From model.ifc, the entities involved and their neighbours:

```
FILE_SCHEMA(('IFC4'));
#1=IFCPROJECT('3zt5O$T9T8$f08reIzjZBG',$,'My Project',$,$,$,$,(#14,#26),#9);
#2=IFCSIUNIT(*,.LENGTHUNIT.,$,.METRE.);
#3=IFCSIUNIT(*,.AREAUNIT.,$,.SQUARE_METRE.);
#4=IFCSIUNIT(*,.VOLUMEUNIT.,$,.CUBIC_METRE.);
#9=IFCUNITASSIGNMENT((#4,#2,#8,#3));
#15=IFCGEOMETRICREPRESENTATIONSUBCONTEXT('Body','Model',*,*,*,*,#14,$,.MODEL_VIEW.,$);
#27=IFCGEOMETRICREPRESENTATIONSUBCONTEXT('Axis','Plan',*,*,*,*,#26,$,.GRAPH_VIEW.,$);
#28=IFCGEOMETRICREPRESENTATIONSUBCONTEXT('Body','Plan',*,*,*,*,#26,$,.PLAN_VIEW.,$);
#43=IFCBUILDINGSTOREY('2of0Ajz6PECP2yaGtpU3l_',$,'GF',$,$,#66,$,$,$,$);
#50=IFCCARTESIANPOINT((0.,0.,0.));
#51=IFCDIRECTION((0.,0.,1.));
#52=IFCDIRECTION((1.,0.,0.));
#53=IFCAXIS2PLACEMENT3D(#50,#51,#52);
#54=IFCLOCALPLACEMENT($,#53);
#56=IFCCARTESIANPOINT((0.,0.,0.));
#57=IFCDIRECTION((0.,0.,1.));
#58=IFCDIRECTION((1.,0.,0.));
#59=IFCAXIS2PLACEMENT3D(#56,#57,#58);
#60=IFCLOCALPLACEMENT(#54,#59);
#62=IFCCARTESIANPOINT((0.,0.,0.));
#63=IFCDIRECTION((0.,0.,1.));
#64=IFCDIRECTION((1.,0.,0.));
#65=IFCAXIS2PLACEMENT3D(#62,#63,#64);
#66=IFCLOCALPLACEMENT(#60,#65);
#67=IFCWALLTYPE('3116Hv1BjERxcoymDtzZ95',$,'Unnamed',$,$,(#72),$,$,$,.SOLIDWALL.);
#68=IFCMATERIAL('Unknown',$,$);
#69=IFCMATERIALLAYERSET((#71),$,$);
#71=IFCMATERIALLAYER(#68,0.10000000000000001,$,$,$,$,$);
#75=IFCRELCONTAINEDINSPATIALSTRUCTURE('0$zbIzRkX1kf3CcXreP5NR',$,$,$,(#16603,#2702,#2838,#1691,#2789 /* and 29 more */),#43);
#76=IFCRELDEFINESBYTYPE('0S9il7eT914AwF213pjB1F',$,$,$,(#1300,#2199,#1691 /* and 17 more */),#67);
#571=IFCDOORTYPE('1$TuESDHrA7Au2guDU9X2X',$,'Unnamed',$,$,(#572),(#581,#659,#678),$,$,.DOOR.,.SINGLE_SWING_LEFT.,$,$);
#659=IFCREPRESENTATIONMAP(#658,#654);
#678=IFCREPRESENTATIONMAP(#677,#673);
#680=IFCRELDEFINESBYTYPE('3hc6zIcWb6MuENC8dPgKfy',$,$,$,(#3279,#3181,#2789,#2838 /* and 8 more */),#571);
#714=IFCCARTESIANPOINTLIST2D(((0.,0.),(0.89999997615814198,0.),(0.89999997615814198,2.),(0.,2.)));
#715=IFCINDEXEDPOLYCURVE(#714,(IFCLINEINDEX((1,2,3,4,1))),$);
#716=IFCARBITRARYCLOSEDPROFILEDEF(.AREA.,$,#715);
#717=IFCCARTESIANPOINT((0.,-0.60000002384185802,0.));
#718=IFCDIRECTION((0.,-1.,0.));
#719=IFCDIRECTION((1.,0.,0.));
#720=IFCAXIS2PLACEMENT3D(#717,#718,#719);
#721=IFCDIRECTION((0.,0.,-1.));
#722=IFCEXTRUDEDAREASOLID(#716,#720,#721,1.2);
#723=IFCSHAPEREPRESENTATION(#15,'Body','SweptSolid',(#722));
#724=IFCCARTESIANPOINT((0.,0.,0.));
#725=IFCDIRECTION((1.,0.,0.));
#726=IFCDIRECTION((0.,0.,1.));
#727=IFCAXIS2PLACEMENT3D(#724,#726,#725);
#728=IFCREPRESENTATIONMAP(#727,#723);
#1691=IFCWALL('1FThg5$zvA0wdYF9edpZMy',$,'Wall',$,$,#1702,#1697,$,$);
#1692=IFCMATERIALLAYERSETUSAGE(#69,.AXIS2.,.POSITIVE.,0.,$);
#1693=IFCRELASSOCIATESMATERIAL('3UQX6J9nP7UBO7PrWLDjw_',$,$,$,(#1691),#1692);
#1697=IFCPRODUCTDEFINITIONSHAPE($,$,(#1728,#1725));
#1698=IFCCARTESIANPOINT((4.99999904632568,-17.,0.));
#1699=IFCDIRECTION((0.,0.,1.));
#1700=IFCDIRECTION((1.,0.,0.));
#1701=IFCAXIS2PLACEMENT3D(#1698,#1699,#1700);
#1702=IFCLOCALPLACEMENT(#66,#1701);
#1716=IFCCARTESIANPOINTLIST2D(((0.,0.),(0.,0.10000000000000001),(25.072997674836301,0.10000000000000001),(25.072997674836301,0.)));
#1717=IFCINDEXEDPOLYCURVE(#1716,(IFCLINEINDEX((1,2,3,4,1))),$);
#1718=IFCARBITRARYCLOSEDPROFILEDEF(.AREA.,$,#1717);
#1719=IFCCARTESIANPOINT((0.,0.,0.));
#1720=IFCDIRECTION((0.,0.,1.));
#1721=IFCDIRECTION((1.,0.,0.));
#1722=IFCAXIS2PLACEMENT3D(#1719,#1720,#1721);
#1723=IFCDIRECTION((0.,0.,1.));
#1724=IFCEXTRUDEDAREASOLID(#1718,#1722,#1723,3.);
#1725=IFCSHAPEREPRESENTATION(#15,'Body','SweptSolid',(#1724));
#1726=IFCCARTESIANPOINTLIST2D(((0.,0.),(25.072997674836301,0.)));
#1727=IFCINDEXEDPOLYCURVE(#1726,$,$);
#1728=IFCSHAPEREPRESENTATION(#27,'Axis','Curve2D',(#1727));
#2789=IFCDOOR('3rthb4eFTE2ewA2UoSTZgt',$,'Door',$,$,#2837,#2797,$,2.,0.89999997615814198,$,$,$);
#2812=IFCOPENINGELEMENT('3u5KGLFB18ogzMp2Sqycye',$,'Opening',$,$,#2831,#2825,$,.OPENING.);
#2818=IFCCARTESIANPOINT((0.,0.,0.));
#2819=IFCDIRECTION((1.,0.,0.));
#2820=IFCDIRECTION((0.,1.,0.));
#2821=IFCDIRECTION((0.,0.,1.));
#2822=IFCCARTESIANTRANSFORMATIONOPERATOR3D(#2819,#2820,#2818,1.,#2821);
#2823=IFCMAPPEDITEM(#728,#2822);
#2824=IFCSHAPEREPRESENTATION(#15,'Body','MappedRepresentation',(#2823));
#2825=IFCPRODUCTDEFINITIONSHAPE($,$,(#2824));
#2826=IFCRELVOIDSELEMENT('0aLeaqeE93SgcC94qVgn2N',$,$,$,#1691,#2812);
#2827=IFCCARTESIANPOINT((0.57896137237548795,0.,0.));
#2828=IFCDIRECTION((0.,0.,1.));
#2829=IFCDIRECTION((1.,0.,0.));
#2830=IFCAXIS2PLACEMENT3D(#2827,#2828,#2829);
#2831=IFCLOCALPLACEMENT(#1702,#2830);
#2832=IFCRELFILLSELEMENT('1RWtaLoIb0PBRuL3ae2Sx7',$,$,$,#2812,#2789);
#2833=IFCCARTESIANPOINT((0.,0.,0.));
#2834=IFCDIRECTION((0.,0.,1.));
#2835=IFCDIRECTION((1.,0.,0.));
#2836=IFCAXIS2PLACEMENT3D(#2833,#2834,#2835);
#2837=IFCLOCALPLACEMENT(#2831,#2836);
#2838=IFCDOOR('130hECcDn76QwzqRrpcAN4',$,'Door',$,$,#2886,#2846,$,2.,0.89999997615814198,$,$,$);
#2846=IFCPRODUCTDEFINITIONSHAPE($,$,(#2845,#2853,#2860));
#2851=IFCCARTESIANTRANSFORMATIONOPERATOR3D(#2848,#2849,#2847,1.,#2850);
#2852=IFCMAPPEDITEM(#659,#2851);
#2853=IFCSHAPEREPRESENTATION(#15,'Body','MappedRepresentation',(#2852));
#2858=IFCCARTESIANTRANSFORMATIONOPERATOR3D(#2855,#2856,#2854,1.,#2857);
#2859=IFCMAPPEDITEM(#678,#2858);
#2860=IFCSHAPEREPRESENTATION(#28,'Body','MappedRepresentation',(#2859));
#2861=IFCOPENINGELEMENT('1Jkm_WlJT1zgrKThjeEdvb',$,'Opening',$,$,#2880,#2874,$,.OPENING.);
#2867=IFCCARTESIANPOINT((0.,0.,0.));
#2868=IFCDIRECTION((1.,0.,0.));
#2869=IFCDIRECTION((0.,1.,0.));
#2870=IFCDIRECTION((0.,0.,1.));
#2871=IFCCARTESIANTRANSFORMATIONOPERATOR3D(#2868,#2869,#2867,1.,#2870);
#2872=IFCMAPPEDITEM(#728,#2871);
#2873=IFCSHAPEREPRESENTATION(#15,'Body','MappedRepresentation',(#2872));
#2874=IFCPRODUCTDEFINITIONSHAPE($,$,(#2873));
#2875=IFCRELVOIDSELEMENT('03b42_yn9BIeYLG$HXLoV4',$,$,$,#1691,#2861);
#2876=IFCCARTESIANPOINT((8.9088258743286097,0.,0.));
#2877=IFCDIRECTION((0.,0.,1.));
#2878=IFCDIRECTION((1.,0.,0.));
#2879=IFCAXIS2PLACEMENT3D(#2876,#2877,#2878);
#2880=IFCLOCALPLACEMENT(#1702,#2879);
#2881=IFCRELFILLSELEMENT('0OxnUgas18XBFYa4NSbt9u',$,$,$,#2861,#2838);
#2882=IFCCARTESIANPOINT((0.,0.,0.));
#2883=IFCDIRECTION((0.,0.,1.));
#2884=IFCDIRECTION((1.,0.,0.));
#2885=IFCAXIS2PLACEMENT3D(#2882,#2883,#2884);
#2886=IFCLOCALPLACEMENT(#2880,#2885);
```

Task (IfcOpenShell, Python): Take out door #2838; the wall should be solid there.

```python
import ifcopenshell
import ifcopenshell.api.feature
import ifcopenshell.api.root
import ifcopenshell.geom
import ifcopenshell.util.shape

model = ifcopenshell.open("model.ifc")
settings = ifcopenshell.geom.settings()


def volume(element):
    """Net volume in cubic metres, openings subtracted."""
    shape = ifcopenshell.geom.create_shape(settings, element)
    return ifcopenshell.util.shape.get_volume(shape.geometry)


door = model.by_guid("130hECcDn76QwzqRrpcAN4")
opening = door.FillsVoids[0].RelatingOpeningElement
wall = opening.VoidsElements[0].RelatingBuildingElement
before = volume(wall)

ifcopenshell.api.root.remove_product(model, product=door)
ifcopenshell.api.feature.remove_feature(model, feature=opening)

after = volume(wall)

print(f"wall volume {before:.3f} -> {after:.3f} m3")

model.write("model_v2.ifc")
```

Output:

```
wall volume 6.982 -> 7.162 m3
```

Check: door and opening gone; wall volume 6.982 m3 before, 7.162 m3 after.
